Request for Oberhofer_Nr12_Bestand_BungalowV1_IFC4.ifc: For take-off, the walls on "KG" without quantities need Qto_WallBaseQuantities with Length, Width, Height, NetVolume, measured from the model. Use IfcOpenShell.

First a look at what the model holds.

```python
import ifcopenshell
import ifcopenshell.util.element
import ifcopenshell.util.unit

model = ifcopenshell.open("Oberhofer_Nr12_Bestand_BungalowV1_IFC4.ifc")
print(model.schema)
for unit_type in ("LENGTHUNIT", "AREAUNIT", "VOLUMEUNIT"):
    print(unit_type, ifcopenshell.util.unit.calculate_unit_scale(model, unit_type))
storey = next(s for s in model.by_type("IfcBuildingStorey") if s.Name == "KG")
walls = [e for e in ifcopenshell.util.element.get_decomposition(storey) if e.is_a("IfcWall")]
for e in sorted(walls, key=lambda e: e.id()):
    print(e.id(), e.is_a(), e.Name, list(ifcopenshell.util.element.get_psets(e, qtos_only=True)), sep=" | ")
```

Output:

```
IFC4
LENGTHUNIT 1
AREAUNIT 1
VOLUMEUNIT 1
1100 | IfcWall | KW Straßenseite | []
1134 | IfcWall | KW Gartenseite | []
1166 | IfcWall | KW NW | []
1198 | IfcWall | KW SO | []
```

```python
import ifcopenshell
import ifcopenshell.api.pset
import ifcopenshell.geom
import ifcopenshell.util.element
import ifcopenshell.util.shape
import ifcopenshell.util.unit

model = ifcopenshell.open("Oberhofer_Nr12_Bestand_BungalowV1_IFC4.ifc")
unit_scale = ifcopenshell.util.unit.calculate_unit_scale(model)
volume_scale = ifcopenshell.util.unit.calculate_unit_scale(model, "VOLUMEUNIT")
settings = ifcopenshell.geom.settings()

storey = next(s for s in model.by_type("IfcBuildingStorey") if s.Name == "KG")
walls = [e for e in ifcopenshell.util.element.get_decomposition(storey) if e.is_a("IfcWall")]

for e in sorted(walls, key=lambda e: e.id()):
    if ifcopenshell.util.element.get_psets(e, qtos_only=True, should_inherit=False):
        continue
    # Geometry comes back in metres, in the element's own axes.
    shape = ifcopenshell.geom.create_shape(settings, e)
    values = {
        "Length": ifcopenshell.util.shape.get_x(shape.geometry) / unit_scale,
        "Width": ifcopenshell.util.shape.get_y(shape.geometry) / unit_scale,
        "Height": ifcopenshell.util.shape.get_z(shape.geometry) / unit_scale,
        "NetVolume": ifcopenshell.util.shape.get_volume(shape.geometry) / volume_scale,
    }
    qto = ifcopenshell.api.pset.add_qto(model, product=e, name="Qto_WallBaseQuantities")
    ifcopenshell.api.pset.edit_qto(model, qto=qto, properties=values)
    print(e.id(), {k: round(v, 3) for k, v in values.items()})

model.write("Oberhofer_Nr12_Bestand_BungalowV1_IFC4_rev.ifc")
```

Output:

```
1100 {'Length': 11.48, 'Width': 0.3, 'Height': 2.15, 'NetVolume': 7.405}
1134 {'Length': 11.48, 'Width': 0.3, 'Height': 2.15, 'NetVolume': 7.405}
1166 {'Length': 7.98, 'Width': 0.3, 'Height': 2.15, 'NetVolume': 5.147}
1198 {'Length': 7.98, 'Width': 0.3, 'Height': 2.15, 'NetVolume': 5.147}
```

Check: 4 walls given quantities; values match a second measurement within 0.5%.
